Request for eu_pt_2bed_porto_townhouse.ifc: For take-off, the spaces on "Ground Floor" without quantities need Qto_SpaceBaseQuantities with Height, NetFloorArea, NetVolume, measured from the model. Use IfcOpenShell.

First a look at what the model holds.

```python
import ifcopenshell
import ifcopenshell.util.element
import ifcopenshell.util.unit

model = ifcopenshell.open("eu_pt_2bed_porto_townhouse.ifc")
print(model.schema)
for unit_type in ("LENGTHUNIT", "AREAUNIT", "VOLUMEUNIT"):
    print(unit_type, ifcopenshell.util.unit.calculate_unit_scale(model, unit_type))
storey = next(s for s in model.by_type("IfcBuildingStorey") if s.Name == "Ground Floor")
spaces = [e for e in ifcopenshell.util.element.get_decomposition(storey) if e.is_a("IfcSpace")]
for e in sorted(spaces, key=lambda e: e.id()):
    print(e.id(), e.is_a(), e.Name, list(ifcopenshell.util.element.get_psets(e, qtos_only=True)), sep=" | ")
```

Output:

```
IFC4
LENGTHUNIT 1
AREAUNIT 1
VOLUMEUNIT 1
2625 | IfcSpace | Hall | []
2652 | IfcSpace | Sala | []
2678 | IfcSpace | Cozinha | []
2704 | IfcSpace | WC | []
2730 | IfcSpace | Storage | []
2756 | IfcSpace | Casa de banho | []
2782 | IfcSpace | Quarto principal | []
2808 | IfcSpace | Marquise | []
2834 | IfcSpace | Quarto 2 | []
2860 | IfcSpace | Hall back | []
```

```python
import ifcopenshell
import ifcopenshell.api.pset
import ifcopenshell.geom
import ifcopenshell.util.element
import ifcopenshell.util.shape
import ifcopenshell.util.unit

model = ifcopenshell.open("eu_pt_2bed_porto_townhouse.ifc")
unit_scale = ifcopenshell.util.unit.calculate_unit_scale(model)
area_scale = ifcopenshell.util.unit.calculate_unit_scale(model, "AREAUNIT")
volume_scale = ifcopenshell.util.unit.calculate_unit_scale(model, "VOLUMEUNIT")
settings = ifcopenshell.geom.settings()

storey = next(s for s in model.by_type("IfcBuildingStorey") if s.Name == "Ground Floor")
spaces = [e for e in ifcopenshell.util.element.get_decomposition(storey) if e.is_a("IfcSpace")]

for e in sorted(spaces, key=lambda e: e.id()):
    if ifcopenshell.util.element.get_psets(e, qtos_only=True, should_inherit=False):
        continue
    # Geometry comes back in metres, in the element's own axes.
    shape = ifcopenshell.geom.create_shape(settings, e)
    values = {
        "Height": ifcopenshell.util.shape.get_z(shape.geometry) / unit_scale,
        "NetFloorArea": ifcopenshell.util.shape.get_footprint_area(shape.geometry) / area_scale,
        "NetVolume": ifcopenshell.util.shape.get_volume(shape.geometry) / volume_scale,
    }
    qto = ifcopenshell.api.pset.add_qto(model, product=e, name="Qto_SpaceBaseQuantities")
    ifcopenshell.api.pset.edit_qto(model, qto=qto, properties=values)
    print(e.id(), {k: round(v, 3) for k, v in values.items()})

model.write("eu_pt_2bed_porto_townhouse_rev.ifc")
```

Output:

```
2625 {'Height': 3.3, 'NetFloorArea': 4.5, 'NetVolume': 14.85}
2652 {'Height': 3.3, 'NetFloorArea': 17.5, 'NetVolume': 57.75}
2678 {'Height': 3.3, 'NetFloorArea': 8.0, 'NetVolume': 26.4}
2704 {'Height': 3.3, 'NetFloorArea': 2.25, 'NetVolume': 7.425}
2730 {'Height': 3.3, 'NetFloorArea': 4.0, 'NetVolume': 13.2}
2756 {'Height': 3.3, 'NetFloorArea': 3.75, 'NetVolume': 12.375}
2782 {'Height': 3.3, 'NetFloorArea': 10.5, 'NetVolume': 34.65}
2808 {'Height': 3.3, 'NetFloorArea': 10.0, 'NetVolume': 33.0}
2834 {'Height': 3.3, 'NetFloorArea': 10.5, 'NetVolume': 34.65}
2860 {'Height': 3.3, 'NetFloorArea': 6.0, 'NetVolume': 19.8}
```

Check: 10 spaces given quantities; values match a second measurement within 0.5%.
